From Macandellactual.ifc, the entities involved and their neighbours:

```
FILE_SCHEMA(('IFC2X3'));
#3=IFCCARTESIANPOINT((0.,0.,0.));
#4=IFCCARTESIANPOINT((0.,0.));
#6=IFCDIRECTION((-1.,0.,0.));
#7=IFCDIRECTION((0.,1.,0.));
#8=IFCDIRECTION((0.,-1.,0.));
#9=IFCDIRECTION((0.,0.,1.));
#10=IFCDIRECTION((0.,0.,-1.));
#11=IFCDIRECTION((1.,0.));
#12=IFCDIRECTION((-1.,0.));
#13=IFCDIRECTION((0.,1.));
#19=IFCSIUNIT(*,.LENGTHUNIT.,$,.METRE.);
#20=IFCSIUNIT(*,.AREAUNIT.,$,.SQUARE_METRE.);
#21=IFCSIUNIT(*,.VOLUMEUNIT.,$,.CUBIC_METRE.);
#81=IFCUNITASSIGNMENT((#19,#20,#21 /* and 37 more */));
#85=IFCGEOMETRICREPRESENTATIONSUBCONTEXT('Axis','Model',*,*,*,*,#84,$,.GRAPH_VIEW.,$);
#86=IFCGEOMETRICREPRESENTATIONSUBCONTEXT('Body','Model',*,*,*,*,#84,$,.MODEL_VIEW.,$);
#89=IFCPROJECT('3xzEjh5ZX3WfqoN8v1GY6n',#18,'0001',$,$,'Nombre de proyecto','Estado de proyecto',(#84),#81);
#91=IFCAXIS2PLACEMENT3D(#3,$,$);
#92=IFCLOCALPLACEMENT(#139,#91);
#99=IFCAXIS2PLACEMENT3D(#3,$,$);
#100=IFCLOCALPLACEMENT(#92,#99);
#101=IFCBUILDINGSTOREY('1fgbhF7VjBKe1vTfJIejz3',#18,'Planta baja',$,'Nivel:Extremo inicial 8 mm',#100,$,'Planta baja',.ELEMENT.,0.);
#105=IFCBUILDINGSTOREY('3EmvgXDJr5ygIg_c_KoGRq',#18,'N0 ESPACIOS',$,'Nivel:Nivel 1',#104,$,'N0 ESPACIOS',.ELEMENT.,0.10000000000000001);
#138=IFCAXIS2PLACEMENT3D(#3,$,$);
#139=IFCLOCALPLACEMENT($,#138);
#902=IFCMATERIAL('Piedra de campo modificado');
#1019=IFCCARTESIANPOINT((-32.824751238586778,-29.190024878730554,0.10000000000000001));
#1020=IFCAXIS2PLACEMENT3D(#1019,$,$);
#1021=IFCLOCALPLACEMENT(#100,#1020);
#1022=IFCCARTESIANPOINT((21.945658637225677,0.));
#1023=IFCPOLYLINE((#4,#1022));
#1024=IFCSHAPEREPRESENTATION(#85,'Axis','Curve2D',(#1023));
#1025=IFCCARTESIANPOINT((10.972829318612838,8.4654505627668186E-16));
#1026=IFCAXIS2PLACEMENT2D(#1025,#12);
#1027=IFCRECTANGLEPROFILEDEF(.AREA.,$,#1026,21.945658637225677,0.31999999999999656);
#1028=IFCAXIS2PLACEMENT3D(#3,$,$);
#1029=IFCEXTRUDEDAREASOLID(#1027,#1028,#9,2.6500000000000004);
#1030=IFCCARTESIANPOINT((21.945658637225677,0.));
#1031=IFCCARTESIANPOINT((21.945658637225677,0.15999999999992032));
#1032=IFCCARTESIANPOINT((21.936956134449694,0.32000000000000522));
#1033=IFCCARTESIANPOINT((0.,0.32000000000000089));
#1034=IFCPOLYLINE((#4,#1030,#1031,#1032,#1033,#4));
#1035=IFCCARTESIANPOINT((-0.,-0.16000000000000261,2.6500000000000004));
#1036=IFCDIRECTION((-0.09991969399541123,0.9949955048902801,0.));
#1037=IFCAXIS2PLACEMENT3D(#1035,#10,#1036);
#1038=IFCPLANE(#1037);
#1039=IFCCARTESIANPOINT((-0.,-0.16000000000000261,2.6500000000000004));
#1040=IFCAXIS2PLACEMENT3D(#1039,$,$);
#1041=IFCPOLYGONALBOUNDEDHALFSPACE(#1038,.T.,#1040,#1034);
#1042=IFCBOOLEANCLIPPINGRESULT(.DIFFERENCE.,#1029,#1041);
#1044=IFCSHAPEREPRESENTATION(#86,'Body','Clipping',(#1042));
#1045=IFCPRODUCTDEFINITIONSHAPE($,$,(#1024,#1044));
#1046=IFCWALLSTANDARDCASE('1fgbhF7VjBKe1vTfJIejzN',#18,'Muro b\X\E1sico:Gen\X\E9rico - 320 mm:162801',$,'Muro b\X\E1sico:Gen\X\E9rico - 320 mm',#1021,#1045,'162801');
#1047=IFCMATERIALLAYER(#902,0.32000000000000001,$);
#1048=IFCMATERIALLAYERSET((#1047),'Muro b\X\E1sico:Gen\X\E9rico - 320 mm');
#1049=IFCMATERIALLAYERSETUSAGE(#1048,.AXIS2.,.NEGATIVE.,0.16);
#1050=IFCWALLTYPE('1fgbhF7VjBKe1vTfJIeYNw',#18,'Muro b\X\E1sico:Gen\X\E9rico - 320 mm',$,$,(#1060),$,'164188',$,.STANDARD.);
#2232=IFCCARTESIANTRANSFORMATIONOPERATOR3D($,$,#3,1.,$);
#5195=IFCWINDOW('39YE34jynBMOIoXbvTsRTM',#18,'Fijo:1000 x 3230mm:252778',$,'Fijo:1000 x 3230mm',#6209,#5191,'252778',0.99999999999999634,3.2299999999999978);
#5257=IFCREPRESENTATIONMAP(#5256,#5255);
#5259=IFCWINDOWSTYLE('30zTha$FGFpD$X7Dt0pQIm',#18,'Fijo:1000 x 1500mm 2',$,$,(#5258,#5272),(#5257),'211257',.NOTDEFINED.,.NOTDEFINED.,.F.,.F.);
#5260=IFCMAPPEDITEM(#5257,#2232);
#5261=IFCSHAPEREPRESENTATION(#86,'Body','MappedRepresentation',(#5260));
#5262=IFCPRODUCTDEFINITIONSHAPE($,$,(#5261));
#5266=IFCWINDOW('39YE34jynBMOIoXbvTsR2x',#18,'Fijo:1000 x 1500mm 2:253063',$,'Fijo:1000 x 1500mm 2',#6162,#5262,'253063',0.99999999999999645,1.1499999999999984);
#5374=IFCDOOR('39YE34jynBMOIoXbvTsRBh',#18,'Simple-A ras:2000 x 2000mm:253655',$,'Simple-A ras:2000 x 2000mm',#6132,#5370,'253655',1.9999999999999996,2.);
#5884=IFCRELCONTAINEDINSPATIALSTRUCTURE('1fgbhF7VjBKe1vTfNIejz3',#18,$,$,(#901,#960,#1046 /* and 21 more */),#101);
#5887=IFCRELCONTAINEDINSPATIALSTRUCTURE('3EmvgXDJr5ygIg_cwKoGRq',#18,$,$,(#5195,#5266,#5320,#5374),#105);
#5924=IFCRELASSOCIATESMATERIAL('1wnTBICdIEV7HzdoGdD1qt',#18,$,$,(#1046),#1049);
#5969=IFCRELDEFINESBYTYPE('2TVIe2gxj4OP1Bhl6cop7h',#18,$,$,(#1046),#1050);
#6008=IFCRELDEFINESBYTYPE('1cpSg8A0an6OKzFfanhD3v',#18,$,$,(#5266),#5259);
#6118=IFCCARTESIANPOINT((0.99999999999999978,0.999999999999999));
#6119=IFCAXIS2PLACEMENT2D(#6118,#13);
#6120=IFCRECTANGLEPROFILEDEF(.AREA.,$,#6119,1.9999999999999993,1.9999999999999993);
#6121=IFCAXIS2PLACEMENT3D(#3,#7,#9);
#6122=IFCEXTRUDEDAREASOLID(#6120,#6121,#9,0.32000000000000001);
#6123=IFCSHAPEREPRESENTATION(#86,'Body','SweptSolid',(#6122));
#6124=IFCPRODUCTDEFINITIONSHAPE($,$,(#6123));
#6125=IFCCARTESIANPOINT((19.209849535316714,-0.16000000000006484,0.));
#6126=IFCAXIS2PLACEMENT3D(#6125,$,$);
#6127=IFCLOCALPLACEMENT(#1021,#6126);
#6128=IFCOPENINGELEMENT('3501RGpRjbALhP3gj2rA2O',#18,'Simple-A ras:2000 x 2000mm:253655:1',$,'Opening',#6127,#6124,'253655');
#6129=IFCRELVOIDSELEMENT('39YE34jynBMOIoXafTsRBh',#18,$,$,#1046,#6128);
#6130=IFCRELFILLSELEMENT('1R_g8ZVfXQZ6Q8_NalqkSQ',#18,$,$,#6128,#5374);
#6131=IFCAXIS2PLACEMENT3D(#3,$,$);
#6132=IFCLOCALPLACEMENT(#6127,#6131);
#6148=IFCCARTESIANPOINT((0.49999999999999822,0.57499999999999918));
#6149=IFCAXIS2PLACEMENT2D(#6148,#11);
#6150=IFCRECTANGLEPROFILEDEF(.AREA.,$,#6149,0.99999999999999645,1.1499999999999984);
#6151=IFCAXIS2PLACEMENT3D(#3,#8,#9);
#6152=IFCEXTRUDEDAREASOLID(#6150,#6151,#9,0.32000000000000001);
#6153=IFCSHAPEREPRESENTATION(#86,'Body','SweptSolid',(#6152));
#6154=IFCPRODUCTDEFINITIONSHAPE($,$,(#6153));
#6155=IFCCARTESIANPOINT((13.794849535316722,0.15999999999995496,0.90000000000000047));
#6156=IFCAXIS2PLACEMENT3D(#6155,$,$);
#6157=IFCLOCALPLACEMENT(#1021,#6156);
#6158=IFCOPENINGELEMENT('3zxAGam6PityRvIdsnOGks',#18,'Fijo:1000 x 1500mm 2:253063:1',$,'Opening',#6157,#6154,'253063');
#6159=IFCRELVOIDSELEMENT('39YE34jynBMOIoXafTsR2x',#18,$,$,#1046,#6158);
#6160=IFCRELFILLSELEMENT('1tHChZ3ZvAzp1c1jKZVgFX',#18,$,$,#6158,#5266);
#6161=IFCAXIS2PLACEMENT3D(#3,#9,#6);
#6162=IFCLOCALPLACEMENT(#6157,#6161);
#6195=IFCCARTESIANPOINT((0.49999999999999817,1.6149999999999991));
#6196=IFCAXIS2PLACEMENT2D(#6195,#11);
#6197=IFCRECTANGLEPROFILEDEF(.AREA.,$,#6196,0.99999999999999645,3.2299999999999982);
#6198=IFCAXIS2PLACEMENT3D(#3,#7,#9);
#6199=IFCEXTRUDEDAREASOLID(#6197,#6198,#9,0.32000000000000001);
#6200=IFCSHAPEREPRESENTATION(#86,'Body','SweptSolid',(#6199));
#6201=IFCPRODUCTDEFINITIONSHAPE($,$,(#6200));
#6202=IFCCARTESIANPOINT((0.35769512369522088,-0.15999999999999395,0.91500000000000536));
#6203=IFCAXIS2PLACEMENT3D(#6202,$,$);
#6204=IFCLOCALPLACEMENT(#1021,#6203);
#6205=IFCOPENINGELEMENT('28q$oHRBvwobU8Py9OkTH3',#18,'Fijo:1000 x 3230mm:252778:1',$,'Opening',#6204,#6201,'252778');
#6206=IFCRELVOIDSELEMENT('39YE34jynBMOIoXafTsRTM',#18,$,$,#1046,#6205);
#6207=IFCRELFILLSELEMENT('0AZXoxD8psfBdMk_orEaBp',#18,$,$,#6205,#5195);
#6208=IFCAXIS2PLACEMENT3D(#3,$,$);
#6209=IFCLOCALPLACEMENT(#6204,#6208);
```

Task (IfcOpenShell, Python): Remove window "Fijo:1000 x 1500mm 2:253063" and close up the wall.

```python
import ifcopenshell
import ifcopenshell.api.feature
import ifcopenshell.api.root
import ifcopenshell.geom
import ifcopenshell.util.shape

model = ifcopenshell.open("Macandellactual.ifc")
settings = ifcopenshell.geom.settings()


def volume(element):
    """Net volume in cubic metres, openings subtracted."""
    shape = ifcopenshell.geom.create_shape(settings, element)
    return ifcopenshell.util.shape.get_volume(shape.geometry)


window = model.by_guid("39YE34jynBMOIoXbvTsR2x")
opening = window.FillsVoids[0].RelatingOpeningElement
wall = opening.VoidsElements[0].RelatingBuildingElement
before = volume(wall)

ifcopenshell.api.root.remove_product(model, product=window)
ifcopenshell.api.feature.remove_feature(model, feature=opening)

after = volume(wall)

print(f"wall volume {before:.3f} -> {after:.3f} m3")

model.write("Macandellactual_v2.ifc")
```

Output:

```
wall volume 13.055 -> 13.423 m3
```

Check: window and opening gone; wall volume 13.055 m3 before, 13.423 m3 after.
